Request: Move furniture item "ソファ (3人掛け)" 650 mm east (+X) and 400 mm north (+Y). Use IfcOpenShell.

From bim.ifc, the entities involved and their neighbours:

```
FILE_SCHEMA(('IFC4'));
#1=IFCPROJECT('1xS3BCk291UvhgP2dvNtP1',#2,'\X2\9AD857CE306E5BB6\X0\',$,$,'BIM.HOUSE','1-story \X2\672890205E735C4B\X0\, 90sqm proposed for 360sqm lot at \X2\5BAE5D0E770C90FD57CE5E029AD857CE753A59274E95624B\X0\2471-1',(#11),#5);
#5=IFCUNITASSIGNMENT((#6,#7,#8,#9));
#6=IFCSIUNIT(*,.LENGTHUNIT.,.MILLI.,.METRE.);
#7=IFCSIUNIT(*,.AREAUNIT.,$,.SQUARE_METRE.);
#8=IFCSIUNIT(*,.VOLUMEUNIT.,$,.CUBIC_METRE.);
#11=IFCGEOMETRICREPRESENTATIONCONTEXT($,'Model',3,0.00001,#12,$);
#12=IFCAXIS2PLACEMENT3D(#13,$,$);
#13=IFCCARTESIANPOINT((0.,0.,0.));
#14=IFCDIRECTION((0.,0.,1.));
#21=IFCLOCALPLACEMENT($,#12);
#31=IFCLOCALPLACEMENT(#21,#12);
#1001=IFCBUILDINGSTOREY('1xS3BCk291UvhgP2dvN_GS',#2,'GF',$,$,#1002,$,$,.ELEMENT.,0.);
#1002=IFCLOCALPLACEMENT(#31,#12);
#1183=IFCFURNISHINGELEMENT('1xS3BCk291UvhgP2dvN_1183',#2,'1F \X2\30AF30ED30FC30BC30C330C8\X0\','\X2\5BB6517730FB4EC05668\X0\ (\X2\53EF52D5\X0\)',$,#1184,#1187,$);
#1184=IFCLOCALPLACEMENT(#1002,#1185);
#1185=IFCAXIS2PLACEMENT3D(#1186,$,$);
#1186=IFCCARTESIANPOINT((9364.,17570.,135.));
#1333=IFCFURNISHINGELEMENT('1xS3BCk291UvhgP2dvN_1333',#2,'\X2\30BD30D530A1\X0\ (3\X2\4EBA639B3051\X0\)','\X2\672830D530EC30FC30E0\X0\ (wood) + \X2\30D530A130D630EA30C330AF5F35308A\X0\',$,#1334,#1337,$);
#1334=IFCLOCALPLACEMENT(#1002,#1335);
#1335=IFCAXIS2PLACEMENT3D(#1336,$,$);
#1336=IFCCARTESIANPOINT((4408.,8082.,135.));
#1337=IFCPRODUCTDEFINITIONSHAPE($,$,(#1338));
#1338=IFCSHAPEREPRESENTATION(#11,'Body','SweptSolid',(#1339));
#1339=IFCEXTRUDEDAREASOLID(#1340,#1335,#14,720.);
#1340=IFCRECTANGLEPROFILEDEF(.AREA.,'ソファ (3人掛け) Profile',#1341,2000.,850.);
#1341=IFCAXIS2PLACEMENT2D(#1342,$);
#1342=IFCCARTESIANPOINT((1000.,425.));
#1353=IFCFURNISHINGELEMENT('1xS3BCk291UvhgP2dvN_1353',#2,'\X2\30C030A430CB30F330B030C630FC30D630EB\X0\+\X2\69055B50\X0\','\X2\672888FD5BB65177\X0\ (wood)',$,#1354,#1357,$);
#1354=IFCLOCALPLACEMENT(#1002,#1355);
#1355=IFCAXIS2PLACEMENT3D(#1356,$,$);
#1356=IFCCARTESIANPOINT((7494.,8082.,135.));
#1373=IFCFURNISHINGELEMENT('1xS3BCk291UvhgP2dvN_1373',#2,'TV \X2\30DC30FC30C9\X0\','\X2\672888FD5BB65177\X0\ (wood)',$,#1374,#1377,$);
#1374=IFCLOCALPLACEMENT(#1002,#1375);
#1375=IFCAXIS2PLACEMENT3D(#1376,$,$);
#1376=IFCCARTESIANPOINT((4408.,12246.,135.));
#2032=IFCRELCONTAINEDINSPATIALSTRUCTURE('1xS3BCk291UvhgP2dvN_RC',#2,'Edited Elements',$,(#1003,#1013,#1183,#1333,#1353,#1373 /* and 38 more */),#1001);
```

```python
import ifcopenshell
import ifcopenshell.api.geometry
import ifcopenshell.util.placement

model = ifcopenshell.open("bim.ifc")

item = model.by_guid("1xS3BCk291UvhgP2dvN_1333")
matrix = ifcopenshell.util.placement.get_local_placement(item.ObjectPlacement)
matrix[0, 3] += 650.0
matrix[1, 3] += 400.0
ifcopenshell.api.geometry.edit_object_placement(model, product=item, matrix=matrix, is_si=False)

print(ifcopenshell.util.placement.get_local_placement(item.ObjectPlacement).round(3) + 0.0)

model.write("bim-out.ifc")
```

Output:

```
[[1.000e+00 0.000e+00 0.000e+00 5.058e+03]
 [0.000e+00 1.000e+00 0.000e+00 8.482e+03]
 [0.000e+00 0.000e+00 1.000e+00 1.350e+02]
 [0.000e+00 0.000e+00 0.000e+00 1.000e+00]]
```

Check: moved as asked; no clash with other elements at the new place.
